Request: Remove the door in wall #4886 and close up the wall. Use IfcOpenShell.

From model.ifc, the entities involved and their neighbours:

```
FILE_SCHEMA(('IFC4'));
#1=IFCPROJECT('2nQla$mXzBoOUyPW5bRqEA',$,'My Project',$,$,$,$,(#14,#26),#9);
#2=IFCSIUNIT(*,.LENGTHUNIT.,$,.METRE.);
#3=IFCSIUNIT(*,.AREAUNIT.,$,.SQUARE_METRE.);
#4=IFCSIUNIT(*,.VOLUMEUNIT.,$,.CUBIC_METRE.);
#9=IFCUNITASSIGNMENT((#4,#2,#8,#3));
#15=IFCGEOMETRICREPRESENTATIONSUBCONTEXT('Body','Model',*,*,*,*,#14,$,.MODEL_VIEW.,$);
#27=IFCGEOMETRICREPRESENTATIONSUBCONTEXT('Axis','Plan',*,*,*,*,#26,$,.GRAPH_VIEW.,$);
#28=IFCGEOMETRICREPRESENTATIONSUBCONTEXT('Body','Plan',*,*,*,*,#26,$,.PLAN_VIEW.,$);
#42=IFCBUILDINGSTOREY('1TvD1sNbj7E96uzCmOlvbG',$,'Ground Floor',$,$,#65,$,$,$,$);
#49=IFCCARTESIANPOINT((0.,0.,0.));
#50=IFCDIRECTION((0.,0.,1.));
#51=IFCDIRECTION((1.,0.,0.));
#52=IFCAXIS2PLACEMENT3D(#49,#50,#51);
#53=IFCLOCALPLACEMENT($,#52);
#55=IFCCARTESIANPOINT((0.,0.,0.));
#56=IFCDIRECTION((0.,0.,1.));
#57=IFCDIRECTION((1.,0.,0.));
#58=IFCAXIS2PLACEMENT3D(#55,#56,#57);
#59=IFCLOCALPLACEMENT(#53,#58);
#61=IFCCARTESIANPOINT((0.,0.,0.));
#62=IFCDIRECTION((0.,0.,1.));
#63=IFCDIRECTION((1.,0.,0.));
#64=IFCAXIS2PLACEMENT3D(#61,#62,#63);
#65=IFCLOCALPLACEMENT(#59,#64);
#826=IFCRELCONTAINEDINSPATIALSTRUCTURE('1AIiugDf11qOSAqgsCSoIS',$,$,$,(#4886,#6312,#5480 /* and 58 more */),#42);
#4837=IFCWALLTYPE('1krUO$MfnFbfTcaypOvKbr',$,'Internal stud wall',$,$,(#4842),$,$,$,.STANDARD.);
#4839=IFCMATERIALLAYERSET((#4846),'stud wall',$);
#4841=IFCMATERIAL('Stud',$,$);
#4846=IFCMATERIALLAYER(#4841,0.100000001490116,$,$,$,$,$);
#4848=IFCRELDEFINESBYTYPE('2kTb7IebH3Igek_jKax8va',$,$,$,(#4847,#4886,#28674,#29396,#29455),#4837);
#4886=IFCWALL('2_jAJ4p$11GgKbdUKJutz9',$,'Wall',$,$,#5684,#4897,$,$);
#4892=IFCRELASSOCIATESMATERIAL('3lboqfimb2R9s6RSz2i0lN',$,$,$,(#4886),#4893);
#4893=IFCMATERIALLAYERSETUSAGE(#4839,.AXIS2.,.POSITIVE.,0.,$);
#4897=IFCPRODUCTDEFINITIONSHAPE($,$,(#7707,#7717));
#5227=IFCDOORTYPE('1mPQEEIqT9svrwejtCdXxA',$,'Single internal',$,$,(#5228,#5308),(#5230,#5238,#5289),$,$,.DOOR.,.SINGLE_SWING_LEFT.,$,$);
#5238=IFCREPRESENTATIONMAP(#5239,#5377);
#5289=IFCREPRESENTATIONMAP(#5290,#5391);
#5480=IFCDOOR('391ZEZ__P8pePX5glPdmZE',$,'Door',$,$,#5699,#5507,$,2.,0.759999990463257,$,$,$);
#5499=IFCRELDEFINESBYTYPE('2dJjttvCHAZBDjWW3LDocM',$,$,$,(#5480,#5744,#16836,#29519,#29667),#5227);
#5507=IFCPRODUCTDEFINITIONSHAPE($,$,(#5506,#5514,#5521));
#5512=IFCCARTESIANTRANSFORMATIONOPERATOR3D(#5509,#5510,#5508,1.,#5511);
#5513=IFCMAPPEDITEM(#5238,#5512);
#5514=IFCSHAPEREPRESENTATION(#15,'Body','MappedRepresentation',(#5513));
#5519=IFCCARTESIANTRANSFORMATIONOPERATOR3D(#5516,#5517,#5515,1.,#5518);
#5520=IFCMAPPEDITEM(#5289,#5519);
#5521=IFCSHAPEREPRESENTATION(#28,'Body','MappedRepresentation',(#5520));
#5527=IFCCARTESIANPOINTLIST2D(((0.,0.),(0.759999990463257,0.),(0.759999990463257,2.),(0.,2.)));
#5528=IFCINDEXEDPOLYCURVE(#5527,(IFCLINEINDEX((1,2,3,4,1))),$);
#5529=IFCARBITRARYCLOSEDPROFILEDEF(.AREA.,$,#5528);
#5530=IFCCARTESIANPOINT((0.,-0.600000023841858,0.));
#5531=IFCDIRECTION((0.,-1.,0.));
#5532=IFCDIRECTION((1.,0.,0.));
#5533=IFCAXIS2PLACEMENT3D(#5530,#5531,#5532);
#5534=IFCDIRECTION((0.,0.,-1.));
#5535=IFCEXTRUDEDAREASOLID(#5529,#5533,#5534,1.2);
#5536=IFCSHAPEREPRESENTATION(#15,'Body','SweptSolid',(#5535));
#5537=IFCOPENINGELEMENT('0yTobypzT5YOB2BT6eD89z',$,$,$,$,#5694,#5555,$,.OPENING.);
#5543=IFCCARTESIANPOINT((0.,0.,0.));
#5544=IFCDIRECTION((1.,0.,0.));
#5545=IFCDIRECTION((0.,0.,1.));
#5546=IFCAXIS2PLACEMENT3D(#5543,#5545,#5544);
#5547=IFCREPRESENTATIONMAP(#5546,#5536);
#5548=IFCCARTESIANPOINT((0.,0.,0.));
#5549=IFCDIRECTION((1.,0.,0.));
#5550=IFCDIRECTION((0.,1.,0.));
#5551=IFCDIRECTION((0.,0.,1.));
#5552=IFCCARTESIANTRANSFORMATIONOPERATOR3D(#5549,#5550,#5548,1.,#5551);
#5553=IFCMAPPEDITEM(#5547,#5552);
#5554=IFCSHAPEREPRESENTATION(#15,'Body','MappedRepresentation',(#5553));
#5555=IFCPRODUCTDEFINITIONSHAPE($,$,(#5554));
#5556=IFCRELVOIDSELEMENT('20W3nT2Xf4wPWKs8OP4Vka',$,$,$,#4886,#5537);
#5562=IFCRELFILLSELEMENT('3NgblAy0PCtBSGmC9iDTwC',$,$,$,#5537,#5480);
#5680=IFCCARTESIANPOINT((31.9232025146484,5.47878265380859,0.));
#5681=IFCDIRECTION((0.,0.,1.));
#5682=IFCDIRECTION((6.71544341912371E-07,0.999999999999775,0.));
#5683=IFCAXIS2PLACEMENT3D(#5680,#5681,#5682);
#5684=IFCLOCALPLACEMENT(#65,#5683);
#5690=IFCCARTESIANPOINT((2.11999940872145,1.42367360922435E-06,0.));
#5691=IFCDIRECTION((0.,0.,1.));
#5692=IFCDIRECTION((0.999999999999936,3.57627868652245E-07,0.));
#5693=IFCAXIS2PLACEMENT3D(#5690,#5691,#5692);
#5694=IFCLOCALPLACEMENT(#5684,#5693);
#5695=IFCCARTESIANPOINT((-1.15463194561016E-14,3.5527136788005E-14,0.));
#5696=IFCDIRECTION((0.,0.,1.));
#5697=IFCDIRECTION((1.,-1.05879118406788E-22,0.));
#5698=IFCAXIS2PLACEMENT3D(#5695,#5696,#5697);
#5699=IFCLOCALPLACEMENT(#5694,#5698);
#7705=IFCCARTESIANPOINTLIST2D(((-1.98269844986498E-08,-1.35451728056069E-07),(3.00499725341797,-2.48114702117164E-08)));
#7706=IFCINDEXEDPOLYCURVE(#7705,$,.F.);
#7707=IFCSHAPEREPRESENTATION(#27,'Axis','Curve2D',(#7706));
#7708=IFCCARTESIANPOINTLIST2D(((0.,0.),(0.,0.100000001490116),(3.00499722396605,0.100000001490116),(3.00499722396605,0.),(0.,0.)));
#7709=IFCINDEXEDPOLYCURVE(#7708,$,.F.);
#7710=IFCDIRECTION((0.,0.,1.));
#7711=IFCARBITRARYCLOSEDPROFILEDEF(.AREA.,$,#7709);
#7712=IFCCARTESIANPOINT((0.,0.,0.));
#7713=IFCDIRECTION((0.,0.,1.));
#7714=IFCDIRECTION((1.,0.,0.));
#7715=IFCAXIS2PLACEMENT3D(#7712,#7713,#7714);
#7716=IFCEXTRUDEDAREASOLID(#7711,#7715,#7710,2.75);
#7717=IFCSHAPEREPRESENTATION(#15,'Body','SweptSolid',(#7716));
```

```python
import ifcopenshell
import ifcopenshell.api.feature
import ifcopenshell.api.root
import ifcopenshell.geom
import ifcopenshell.util.shape

model = ifcopenshell.open("model.ifc")
settings = ifcopenshell.geom.settings()


def volume(element):
    """Net volume in cubic metres, openings subtracted."""
    shape = ifcopenshell.geom.create_shape(settings, element)
    return ifcopenshell.util.shape.get_volume(shape.geometry)


door = model.by_guid("391ZEZ__P8pePX5glPdmZE")
opening = door.FillsVoids[0].RelatingOpeningElement
wall = opening.VoidsElements[0].RelatingBuildingElement
before = volume(wall)

ifcopenshell.api.root.remove_product(model, product=door)
ifcopenshell.api.feature.remove_feature(model, feature=opening)

after = volume(wall)

print(f"wall volume {before:.3f} -> {after:.3f} m3")

model.write("model_edited.ifc")
```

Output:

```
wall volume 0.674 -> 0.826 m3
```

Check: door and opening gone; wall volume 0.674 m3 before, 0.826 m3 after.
